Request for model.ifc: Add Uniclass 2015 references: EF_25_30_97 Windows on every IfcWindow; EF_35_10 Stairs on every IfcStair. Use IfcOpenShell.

First a look at what the model holds.

```python
import ifcopenshell

model = ifcopenshell.open("model.ifc")
print(model.schema)
print("classifications:", [c.Name for c in model.by_type("IfcClassification")])
for ifc_class in ("IfcDoor", "IfcRoof", "IfcStair", "IfcWall", "IfcWindow"):
    print(ifc_class, len(model.by_type(ifc_class)))
```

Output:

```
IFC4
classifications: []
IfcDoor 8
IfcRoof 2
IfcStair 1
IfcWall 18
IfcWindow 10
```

```python
import ifcopenshell
import ifcopenshell.api.classification

model = ifcopenshell.open("model.ifc")

system = ifcopenshell.api.classification.add_classification(model, classification="Uniclass 2015")

codes = {
    "IfcWindow": ("EF_25_30_97", "Windows"),
    "IfcStair": ("EF_35_10", "Stairs"),
}
for ifc_class, (code, name) in codes.items():
    products = model.by_type(ifc_class)
    ifcopenshell.api.classification.add_reference(
        model, products=products, classification=system, identification=code, name=name
    )
    print(code, len(products))

model.write("model_v2.ifc")
```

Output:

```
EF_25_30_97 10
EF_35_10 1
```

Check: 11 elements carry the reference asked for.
